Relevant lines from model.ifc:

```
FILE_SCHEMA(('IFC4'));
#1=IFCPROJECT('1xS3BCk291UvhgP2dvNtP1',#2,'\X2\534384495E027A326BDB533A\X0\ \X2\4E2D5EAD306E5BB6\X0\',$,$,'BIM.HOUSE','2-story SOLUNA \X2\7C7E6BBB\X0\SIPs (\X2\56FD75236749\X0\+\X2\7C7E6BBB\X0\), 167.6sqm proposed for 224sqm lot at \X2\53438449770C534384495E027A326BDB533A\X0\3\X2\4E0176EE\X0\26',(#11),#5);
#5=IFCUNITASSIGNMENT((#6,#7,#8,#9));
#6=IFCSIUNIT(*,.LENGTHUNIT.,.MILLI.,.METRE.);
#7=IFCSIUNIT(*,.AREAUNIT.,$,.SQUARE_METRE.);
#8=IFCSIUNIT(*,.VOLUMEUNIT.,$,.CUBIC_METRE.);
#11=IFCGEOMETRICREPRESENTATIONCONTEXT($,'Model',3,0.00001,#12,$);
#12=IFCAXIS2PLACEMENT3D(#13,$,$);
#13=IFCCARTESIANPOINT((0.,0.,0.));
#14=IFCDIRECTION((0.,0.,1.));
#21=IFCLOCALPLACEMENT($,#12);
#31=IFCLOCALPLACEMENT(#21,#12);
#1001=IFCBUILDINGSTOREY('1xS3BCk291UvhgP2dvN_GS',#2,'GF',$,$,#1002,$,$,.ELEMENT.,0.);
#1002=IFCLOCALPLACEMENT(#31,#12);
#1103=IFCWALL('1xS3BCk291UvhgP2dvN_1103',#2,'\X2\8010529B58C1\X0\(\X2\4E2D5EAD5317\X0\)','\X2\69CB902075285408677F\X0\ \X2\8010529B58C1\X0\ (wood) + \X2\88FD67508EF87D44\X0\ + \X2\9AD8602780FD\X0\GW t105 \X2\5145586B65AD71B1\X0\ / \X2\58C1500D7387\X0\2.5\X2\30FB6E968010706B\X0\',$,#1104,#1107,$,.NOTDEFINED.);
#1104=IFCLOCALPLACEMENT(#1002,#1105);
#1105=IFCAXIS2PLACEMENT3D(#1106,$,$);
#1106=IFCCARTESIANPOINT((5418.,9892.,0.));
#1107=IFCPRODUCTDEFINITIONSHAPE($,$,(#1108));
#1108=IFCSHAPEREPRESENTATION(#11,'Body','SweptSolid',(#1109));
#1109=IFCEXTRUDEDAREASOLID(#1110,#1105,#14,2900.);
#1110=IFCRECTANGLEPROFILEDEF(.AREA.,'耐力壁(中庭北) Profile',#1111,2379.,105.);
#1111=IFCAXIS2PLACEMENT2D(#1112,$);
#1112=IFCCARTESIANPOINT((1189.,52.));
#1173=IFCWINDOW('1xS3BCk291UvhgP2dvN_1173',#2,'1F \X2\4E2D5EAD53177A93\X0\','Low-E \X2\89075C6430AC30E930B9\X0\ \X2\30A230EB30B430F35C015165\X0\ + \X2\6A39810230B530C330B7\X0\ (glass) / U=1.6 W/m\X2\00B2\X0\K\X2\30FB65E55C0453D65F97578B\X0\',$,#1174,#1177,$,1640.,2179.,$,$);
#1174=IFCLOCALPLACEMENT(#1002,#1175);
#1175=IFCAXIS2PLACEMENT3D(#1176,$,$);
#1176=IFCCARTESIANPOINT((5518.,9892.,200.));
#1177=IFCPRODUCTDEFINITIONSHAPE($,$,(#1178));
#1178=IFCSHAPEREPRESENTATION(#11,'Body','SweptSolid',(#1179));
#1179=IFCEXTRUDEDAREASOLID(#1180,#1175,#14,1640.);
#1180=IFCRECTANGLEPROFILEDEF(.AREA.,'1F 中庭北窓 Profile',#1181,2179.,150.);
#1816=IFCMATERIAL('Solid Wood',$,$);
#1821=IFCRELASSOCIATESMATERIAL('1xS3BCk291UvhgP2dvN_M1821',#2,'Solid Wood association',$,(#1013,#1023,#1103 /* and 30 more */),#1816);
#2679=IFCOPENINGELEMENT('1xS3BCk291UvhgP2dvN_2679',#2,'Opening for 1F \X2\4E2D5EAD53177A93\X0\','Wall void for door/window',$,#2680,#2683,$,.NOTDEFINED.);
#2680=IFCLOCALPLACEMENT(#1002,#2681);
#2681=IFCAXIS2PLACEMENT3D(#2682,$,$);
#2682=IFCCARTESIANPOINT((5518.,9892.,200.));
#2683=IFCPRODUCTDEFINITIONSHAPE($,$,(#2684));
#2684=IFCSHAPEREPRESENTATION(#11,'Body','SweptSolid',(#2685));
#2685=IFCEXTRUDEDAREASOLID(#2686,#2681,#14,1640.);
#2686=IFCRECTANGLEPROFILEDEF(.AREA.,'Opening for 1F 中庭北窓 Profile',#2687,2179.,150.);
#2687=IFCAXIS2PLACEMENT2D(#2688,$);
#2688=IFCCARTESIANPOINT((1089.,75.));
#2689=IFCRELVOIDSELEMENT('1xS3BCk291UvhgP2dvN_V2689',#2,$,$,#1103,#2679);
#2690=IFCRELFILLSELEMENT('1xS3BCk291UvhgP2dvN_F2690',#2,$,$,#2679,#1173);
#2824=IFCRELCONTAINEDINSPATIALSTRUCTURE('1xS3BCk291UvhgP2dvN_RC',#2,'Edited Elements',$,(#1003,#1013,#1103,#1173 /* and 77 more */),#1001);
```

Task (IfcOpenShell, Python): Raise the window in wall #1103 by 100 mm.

```python
import numpy as np
import ifcopenshell
import ifcopenshell.api.geometry
import ifcopenshell.util.placement
import ifcopenshell.util.unit

model = ifcopenshell.open("model.ifc")
unit_scale = ifcopenshell.util.unit.calculate_unit_scale(model)

window = model.by_guid("1xS3BCk291UvhgP2dvN_1173")
opening = window.FillsVoids[0].RelatingOpeningElement
dz = 0.1 / unit_scale

shift = np.array([0.0, 0.0, dz])
# The window is not placed relative to its opening, so move both.
for product in (opening, window):
    matrix = ifcopenshell.util.placement.get_local_placement(product.ObjectPlacement)
    matrix[:3, 3] += shift
    ifcopenshell.api.geometry.edit_object_placement(model, product=product, matrix=matrix, is_si=False)

print(f"moved by {dz * unit_scale:+.3f} m")

model.write("model_edited.ifc")
```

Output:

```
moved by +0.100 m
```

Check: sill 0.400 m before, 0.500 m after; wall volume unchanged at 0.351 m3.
